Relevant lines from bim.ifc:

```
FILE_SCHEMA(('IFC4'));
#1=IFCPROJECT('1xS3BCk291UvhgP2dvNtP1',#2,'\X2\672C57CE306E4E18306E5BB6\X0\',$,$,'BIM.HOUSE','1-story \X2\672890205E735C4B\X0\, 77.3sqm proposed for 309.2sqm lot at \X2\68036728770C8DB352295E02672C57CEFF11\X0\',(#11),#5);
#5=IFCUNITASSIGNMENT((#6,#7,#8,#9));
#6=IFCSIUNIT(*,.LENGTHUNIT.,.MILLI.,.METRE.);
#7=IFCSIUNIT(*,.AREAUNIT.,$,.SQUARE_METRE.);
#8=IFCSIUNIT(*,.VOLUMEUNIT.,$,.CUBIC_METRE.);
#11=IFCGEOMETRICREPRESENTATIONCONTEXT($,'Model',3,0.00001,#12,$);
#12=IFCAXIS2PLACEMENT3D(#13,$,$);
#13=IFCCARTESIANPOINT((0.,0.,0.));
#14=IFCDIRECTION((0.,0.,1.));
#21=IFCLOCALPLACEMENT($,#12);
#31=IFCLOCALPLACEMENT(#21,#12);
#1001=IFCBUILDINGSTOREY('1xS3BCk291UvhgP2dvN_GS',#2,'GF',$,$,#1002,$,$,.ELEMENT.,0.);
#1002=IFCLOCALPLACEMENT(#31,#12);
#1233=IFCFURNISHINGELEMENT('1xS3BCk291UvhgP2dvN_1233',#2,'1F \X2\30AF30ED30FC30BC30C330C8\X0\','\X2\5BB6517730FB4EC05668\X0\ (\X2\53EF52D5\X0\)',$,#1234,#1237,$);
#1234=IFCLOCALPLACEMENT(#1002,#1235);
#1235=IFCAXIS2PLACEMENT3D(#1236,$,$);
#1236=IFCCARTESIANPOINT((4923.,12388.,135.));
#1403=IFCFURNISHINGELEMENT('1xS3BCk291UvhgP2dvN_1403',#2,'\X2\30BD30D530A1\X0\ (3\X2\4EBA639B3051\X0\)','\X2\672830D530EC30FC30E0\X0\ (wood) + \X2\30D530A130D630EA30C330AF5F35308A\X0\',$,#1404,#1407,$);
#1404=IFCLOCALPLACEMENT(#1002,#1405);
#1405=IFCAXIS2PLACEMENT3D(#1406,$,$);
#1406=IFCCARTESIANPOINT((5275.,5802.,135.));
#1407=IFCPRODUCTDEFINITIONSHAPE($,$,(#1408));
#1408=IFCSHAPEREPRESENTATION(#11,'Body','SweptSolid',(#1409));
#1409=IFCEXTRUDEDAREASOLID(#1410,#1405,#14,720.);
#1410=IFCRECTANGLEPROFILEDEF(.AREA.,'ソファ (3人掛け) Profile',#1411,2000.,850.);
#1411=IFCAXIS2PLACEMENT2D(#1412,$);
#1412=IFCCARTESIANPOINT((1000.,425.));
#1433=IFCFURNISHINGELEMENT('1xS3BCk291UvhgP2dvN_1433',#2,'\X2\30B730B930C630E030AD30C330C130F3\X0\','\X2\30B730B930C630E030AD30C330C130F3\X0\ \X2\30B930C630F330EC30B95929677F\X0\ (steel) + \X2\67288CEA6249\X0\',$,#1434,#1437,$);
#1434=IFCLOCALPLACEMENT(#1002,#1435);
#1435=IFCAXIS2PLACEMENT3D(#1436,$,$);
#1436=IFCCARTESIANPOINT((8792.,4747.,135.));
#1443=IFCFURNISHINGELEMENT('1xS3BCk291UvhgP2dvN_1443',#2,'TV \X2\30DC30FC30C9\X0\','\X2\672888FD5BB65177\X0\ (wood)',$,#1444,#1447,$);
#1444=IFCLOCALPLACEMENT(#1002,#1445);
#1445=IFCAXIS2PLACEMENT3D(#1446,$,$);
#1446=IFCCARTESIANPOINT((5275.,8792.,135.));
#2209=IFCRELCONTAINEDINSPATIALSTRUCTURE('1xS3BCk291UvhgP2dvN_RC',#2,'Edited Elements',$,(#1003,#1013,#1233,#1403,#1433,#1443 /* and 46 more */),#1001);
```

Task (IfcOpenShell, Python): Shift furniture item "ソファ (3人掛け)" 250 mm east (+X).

```python
import ifcopenshell
import ifcopenshell.api.geometry
import ifcopenshell.util.placement
import ifcopenshell.util.unit

model = ifcopenshell.open("bim.ifc")
unit_scale = ifcopenshell.util.unit.calculate_unit_scale(model)

item = model.by_guid("1xS3BCk291UvhgP2dvN_1403")
matrix = ifcopenshell.util.placement.get_local_placement(item.ObjectPlacement)
matrix[0, 3] += 0.25 / unit_scale
ifcopenshell.api.geometry.edit_object_placement(model, product=item, matrix=matrix, is_si=False)

print(ifcopenshell.util.placement.get_local_placement(item.ObjectPlacement).round(3) + 0.0)

model.write("bim-out.ifc")
```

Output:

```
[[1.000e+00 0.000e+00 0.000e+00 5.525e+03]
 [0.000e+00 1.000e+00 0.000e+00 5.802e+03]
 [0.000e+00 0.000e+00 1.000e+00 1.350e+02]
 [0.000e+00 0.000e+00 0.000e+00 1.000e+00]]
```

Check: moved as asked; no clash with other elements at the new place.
